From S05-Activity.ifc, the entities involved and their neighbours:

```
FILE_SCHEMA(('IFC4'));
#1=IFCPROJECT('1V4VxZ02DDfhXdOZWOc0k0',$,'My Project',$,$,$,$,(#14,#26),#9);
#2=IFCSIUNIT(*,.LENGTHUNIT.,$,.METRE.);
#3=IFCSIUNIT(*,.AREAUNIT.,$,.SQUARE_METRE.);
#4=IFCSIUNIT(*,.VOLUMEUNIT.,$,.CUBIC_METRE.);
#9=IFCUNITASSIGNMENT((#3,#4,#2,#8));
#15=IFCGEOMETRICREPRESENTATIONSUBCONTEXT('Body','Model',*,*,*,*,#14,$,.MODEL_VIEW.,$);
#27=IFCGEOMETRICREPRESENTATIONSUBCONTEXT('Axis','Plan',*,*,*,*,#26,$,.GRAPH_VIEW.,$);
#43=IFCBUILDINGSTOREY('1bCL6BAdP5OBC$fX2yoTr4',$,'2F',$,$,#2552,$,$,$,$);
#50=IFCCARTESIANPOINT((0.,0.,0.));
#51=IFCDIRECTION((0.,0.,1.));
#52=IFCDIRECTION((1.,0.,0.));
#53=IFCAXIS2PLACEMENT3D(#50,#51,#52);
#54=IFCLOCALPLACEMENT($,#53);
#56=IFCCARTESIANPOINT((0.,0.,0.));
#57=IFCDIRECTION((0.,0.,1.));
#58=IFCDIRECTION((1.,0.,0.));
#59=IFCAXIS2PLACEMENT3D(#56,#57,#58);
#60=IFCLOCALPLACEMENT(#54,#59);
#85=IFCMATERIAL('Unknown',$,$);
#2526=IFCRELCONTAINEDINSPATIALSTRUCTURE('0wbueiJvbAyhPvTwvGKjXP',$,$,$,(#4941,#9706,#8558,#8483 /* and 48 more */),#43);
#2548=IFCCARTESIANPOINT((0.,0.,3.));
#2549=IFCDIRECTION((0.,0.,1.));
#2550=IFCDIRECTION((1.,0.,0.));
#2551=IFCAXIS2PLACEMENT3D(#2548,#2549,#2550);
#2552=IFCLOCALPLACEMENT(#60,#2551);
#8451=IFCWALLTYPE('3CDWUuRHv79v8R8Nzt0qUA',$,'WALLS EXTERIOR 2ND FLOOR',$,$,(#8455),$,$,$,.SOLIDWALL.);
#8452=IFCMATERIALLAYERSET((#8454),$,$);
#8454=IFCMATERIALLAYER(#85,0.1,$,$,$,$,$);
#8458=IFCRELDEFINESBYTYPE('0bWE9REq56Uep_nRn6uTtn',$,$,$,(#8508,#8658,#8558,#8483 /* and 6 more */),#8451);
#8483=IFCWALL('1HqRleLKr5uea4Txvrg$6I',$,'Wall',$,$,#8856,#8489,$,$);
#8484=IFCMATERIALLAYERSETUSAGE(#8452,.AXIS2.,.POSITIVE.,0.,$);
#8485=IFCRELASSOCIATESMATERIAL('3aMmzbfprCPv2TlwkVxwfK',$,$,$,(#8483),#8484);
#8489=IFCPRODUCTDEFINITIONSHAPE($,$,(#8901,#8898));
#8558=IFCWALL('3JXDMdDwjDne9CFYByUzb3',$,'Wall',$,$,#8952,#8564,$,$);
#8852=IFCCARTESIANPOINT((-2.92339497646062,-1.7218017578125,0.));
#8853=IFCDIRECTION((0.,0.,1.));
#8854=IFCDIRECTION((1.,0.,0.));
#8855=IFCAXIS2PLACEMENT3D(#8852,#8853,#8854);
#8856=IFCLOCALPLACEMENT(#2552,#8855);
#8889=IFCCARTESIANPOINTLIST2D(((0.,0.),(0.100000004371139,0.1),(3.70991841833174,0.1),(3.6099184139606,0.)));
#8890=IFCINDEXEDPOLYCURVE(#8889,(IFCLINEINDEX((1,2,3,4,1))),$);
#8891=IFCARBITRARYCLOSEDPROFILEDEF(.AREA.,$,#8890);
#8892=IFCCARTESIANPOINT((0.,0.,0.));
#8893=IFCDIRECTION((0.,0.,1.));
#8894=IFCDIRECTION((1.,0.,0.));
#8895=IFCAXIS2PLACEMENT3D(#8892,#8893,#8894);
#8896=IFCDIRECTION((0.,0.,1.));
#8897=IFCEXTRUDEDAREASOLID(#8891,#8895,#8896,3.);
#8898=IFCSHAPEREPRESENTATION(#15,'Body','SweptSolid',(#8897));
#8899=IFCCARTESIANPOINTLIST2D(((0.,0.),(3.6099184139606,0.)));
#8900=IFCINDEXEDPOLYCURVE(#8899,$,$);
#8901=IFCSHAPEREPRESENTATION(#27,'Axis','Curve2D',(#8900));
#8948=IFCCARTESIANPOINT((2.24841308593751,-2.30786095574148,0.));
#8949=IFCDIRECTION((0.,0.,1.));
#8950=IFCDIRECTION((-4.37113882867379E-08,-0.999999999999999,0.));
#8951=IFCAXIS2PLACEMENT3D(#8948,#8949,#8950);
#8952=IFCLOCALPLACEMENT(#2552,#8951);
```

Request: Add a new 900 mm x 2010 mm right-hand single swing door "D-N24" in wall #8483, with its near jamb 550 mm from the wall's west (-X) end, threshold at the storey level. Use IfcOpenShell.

```python
import numpy as np
import ifcopenshell
import ifcopenshell.api.feature
import ifcopenshell.api.geometry
import ifcopenshell.api.root
import ifcopenshell.api.spatial
import ifcopenshell.geom
import ifcopenshell.util.element
import ifcopenshell.util.placement
import ifcopenshell.util.representation
import ifcopenshell.util.shape
import ifcopenshell.util.unit

model = ifcopenshell.open("S05-Activity.ifc")
unit_scale = ifcopenshell.util.unit.calculate_unit_scale(model)
settings = ifcopenshell.geom.settings()


def volume(element):
    """Net volume in cubic metres, openings subtracted."""
    shape = ifcopenshell.geom.create_shape(settings, element)
    return ifcopenshell.util.shape.get_volume(shape.geometry)


wall = model.by_id(8483)
storey = ifcopenshell.util.element.get_container(wall, ifc_class="IfcBuildingStorey")
context = ifcopenshell.util.representation.get_context(model, "Model", "Body", "MODEL_VIEW")
before = volume(wall)

width, height, from_end, sill = 0.9, 2.01, 0.55, 0.0  # metres

# The wall runs along its own X axis, and the end named is its -X end.
wall_shape = ifcopenshell.geom.create_shape(settings, wall)
x, y, z = ifcopenshell.util.shape.get_vertices(wall_shape.geometry).T
start = x.min() + from_end
face, thickness = float(y.min()), float(y.max() - y.min())
wall_matrix = ifcopenshell.util.placement.get_local_placement(wall.ObjectPlacement)
level = ifcopenshell.util.placement.get_local_placement(storey.ObjectPlacement)[2, 3]


def in_wall(x, y):
    """Placement at x, y metres in the wall's axes, at sill height."""
    matrix = wall_matrix.copy()
    matrix[:, 3] = wall_matrix @ np.array([x / unit_scale, y / unit_scale, 0.0, 1.0])
    matrix[2, 3] = level + sill / unit_scale
    return matrix


# Opening: a box that overshoots both wall faces by 50 mm.
opening = ifcopenshell.api.root.create_entity(model, ifc_class="IfcOpeningElement", predefined_type="OPENING")
box = ifcopenshell.api.geometry.add_wall_representation(
    model, context=context, length=width, height=height, thickness=thickness + 0.1
)
ifcopenshell.api.geometry.assign_representation(model, product=opening, representation=box)
ifcopenshell.api.geometry.edit_object_placement(model, product=opening, matrix=in_wall(start, face - 0.05), is_si=False)
ifcopenshell.api.feature.add_feature(model, feature=opening, element=wall)

door = ifcopenshell.api.root.create_entity(model, ifc_class="IfcDoor", name="D-N24", predefined_type="DOOR")
door.OverallWidth, door.OverallHeight = width / unit_scale, height / unit_scale
door.OperationType = "SINGLE_SWING_RIGHT"
body = ifcopenshell.api.geometry.add_door_representation(
    model,
    context=context,
    overall_width=door.OverallWidth,
    overall_height=door.OverallHeight,
    operation_type="SINGLE_SWING_RIGHT",
    lining_properties={"LiningDepth": thickness / unit_scale, "ThresholdDepth": thickness / unit_scale},
)
ifcopenshell.api.geometry.assign_representation(model, product=door, representation=body)
ifcopenshell.api.spatial.assign_container(model, products=[door], relating_structure=storey)
ifcopenshell.api.feature.add_filling(model, opening=opening, element=door)

# The lining spans the wall, so the door starts at the wall face.
ifcopenshell.api.geometry.edit_object_placement(model, product=door, matrix=in_wall(start, face), is_si=False)

after = volume(wall)

print(f"wall volume {before:.3f} -> {after:.3f} m3")

model.write("S05-Activity_edited.ifc")
```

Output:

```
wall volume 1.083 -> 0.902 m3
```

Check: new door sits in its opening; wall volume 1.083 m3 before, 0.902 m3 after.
